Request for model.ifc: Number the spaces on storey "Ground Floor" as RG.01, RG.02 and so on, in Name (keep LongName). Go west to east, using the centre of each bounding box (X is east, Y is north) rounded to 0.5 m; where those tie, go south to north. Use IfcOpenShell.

First a look at what the model holds.

```python
import ifcopenshell
import ifcopenshell.util.element
import ifcopenshell.util.placement

model = ifcopenshell.open("model.ifc")
print(model.schema)
storey = next(s for s in model.by_type("IfcBuildingStorey") if s.Name == "Ground Floor")
spaces = [e for e in ifcopenshell.util.element.get_decomposition(storey) if e.is_a("IfcSpace")]
for e in sorted(spaces, key=lambda e: e.id()):
    origin = ifcopenshell.util.placement.get_local_placement(e.ObjectPlacement)[:3, 3]
    print(e.id(), e.Name, e.LongName, origin.round(2) + 0.0, sep=" | ")
```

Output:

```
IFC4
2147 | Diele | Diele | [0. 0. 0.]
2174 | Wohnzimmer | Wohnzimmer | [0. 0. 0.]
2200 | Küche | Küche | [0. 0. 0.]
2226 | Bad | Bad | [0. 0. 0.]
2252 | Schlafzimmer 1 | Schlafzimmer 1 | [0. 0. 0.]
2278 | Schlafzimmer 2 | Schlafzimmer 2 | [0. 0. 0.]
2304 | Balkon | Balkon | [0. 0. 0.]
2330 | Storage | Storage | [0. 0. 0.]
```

```python
import ifcopenshell
import ifcopenshell.geom
import ifcopenshell.util.element
import ifcopenshell.util.shape

model = ifcopenshell.open("model.ifc")
settings = ifcopenshell.geom.settings()
settings.set("use-world-coords", True)


def centre(element):
    shape = ifcopenshell.geom.create_shape(settings, element)
    return ifcopenshell.util.shape.get_bbox_centroid(shape.geometry)


storey = next(s for s in model.by_type("IfcBuildingStorey") if s.Name == "Ground Floor")
spaces = [e for e in ifcopenshell.util.element.get_decomposition(storey) if e.is_a("IfcSpace")]

# Insertion points can sit at a corner or the storey origin, so sort by the geometry (in metres).
centres = {e: centre(e) for e in spaces}
spaces.sort(key=lambda e: (round(centres[e][0] / 0.5), centres[e][1]))

for i, e in enumerate(spaces, start=1):
    number = f"RG.{i:02d}"
    e.Name = number
    print(e.id(), number)

model.write("model-out.ifc")
```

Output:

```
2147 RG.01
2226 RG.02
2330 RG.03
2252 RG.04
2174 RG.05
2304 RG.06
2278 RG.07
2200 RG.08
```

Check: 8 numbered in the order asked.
